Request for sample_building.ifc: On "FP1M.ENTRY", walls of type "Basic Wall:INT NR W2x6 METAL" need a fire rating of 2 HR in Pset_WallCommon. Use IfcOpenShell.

First a look at what the model holds.

```python
import ifcopenshell
import ifcopenshell.util.element

model = ifcopenshell.open("sample_building.ifc")
print(model.schema)
storey = next(s for s in model.by_type("IfcBuildingStorey") if s.Name == "FP1M.ENTRY")
walls = [e for e in ifcopenshell.util.element.get_decomposition(storey) if e.is_a("IfcWall")]
seen = {}
for e in walls:
    element_type = ifcopenshell.util.element.get_type(e)
    key = (element_type.Name if element_type != e and element_type else None, ifcopenshell.util.element.get_pset(e, "Pset_WallCommon", "FireRating"))
    seen[key] = seen.get(key, 0) + 1
for (name, value), count in sorted(seen.items(), key=str):
    print(count, "x", name, "|", value)
```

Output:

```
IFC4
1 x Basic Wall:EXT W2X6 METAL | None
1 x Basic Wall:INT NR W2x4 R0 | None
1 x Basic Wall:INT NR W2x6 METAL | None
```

```python
import ifcopenshell
import ifcopenshell.api.pset
import ifcopenshell.util.element

model = ifcopenshell.open("sample_building.ifc")

storey = next(s for s in model.by_type("IfcBuildingStorey") if s.Name == "FP1M.ENTRY")
walls = [e for e in ifcopenshell.util.element.get_decomposition(storey) if e.is_a("IfcWall")]

count = 0
for e in walls:
    element_type = ifcopenshell.util.element.get_type(e)
    if element_type in (None, e) or element_type.Name != "Basic Wall:INT NR W2x6 METAL":
        continue
    # add_pset returns the element's existing set when there is one.
    pset = ifcopenshell.api.pset.add_pset(model, product=e, name="Pset_WallCommon")
    ifcopenshell.api.pset.edit_pset(model, pset=pset, properties={"FireRating": "2 HR"})
    count += 1

print(count, "walls updated")

model.write("sample_building_updated.ifc")
```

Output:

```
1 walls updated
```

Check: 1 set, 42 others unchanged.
